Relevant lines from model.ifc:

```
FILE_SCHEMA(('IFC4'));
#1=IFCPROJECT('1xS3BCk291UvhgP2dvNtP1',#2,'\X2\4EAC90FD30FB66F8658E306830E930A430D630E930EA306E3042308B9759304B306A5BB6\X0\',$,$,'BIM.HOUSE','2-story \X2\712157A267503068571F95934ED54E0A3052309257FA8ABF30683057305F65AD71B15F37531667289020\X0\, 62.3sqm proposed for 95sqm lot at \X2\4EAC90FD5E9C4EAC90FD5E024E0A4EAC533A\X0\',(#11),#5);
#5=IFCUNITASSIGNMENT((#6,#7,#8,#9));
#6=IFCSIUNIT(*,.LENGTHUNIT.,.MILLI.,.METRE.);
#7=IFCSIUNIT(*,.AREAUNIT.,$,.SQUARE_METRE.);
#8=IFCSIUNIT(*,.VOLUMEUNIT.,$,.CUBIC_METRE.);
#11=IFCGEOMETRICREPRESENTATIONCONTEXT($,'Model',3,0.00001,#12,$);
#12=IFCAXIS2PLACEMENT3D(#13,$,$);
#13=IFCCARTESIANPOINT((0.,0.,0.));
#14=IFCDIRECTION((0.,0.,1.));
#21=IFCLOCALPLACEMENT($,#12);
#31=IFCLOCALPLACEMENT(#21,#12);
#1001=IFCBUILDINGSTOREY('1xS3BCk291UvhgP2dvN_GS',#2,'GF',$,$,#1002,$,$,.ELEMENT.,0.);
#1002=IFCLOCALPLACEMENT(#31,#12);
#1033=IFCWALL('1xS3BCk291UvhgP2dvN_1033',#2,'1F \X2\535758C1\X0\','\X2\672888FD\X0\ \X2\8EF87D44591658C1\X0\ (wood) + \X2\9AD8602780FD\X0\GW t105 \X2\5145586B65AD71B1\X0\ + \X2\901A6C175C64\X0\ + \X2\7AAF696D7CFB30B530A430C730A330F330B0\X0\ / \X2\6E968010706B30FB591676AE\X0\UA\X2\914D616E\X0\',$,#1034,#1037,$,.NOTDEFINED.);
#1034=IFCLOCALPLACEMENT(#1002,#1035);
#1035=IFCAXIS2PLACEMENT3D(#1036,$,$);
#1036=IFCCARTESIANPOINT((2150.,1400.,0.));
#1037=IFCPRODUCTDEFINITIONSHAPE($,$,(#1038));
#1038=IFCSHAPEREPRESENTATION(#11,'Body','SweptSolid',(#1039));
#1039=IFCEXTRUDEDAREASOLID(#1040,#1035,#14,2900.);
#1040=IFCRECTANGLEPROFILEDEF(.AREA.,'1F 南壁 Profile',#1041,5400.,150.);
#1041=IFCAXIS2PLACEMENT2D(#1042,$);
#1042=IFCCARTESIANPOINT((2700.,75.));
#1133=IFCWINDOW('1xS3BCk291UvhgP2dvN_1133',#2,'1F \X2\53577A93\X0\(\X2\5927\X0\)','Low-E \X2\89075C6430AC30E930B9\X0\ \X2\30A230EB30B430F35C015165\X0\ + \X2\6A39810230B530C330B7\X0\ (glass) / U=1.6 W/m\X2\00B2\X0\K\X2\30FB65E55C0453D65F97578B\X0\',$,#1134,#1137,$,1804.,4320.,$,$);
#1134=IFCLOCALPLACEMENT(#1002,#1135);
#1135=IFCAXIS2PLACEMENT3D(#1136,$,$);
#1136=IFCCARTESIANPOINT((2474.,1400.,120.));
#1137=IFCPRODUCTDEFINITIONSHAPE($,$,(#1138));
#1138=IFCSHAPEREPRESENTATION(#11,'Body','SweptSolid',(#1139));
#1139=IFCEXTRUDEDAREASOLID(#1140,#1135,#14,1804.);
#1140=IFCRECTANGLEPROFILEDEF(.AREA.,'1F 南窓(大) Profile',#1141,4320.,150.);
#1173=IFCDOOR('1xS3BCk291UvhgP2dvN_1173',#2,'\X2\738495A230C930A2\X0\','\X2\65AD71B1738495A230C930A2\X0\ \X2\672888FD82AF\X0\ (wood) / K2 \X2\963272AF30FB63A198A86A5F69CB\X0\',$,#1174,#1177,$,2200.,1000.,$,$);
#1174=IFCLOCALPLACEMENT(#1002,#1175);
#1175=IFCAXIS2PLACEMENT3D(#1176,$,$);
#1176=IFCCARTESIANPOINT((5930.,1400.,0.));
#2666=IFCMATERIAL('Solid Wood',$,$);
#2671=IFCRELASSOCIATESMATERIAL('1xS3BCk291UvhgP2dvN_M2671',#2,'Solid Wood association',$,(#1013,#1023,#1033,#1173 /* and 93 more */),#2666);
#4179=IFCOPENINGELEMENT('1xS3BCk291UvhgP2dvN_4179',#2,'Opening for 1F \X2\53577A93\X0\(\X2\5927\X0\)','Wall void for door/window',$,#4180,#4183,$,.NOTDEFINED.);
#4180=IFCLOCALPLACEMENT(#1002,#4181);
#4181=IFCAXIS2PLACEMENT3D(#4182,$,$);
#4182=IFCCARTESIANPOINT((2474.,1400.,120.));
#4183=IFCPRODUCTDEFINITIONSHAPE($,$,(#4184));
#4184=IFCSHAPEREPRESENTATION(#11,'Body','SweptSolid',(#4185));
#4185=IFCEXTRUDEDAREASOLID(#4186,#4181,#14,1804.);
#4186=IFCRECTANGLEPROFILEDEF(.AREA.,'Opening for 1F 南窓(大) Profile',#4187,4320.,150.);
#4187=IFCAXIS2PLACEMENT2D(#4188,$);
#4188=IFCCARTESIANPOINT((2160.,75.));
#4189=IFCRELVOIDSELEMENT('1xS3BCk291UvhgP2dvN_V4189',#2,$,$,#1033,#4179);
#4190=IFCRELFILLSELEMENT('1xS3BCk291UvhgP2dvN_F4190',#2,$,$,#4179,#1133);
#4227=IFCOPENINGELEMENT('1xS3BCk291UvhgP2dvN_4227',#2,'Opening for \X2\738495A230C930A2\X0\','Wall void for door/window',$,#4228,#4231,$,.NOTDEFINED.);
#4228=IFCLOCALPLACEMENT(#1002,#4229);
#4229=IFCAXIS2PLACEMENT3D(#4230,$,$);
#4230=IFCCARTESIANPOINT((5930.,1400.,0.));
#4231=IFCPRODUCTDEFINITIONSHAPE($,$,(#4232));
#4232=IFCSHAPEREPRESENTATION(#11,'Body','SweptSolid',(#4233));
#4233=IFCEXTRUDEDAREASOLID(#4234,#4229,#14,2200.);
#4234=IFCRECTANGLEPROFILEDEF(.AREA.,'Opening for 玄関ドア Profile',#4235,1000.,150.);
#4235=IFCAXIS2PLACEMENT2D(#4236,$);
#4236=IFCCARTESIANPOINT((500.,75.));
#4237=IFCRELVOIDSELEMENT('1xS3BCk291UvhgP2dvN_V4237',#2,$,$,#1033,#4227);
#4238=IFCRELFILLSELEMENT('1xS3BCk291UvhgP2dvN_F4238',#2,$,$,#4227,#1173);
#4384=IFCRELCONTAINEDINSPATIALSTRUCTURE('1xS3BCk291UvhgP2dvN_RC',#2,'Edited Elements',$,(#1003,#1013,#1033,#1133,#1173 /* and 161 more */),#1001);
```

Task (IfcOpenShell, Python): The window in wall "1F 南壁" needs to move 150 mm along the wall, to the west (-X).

```python
import ifcopenshell
import ifcopenshell.api.geometry
import ifcopenshell.util.placement
import ifcopenshell.util.unit

model = ifcopenshell.open("model.ifc")
unit_scale = ifcopenshell.util.unit.calculate_unit_scale(model)

window = model.by_id(1133)
opening = window.FillsVoids[0].RelatingOpeningElement
wall = opening.VoidsElements[0].RelatingBuildingElement

wall_matrix = ifcopenshell.util.placement.get_local_placement(wall.ObjectPlacement)
shift = wall_matrix[:3, 0] * -0.15 / unit_scale
before = ifcopenshell.util.placement.get_local_placement(window.ObjectPlacement)[:3, 3].copy()

# The window is not placed relative to its opening, so move both.
for product in (opening, window):
    matrix = ifcopenshell.util.placement.get_local_placement(product.ObjectPlacement)
    matrix[:3, 3] += shift
    ifcopenshell.api.geometry.edit_object_placement(model, product=product, matrix=matrix, is_si=False)

after = ifcopenshell.util.placement.get_local_placement(window.ObjectPlacement)[:3, 3]
print("window moved by", (after - before).round(3) + 0.0)

model.write("model_v2.ifc")
```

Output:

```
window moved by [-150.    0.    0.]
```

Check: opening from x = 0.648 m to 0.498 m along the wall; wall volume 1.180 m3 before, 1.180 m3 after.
